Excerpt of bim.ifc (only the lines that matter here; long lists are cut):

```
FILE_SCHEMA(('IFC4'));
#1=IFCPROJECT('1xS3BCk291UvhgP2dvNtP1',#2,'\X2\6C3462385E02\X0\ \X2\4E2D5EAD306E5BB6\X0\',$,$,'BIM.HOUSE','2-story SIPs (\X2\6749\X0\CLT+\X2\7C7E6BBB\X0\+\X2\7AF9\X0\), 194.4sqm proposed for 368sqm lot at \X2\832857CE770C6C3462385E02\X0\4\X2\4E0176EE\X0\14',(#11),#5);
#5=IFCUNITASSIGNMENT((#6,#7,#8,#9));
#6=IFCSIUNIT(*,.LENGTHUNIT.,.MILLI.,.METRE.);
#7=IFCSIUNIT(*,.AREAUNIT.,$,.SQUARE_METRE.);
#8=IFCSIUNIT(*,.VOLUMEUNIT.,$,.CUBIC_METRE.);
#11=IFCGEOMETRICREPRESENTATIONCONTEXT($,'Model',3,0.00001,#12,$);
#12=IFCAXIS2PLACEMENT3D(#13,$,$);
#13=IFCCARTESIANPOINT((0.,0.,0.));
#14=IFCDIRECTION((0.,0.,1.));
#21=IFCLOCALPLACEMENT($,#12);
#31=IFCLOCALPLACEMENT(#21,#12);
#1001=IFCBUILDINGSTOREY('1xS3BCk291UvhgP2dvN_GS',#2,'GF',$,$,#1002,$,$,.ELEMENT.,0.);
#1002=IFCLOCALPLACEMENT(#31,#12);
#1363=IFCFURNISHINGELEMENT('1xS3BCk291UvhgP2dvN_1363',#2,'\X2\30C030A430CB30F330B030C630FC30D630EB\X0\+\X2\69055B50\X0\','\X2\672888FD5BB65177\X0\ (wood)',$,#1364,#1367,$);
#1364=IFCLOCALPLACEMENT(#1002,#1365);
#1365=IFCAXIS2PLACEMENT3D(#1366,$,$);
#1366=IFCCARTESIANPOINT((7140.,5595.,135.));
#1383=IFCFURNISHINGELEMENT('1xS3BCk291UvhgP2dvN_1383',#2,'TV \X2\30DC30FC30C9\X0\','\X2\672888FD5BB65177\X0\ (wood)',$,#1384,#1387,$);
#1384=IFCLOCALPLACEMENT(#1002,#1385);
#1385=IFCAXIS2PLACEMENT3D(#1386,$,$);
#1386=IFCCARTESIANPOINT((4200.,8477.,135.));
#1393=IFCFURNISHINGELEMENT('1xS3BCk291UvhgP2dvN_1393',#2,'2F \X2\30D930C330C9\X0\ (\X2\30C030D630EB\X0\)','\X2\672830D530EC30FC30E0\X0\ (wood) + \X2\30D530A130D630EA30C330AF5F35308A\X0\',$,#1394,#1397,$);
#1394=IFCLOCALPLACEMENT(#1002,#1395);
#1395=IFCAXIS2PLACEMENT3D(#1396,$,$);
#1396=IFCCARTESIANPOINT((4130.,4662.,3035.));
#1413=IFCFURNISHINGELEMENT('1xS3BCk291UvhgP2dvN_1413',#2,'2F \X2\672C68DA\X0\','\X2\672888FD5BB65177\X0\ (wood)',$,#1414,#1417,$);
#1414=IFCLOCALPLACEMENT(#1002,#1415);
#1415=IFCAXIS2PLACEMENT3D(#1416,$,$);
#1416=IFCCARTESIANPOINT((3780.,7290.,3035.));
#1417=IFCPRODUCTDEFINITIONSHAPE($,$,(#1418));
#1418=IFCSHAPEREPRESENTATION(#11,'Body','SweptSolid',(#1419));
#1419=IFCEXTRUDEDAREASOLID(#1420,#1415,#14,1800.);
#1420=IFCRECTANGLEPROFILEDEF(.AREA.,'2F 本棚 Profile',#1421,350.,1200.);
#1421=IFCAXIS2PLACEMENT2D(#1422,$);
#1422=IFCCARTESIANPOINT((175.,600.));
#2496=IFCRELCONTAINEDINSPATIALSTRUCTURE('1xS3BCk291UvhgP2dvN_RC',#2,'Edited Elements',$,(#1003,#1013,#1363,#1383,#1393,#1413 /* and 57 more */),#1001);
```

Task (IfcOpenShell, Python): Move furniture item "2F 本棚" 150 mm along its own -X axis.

```python
import ifcopenshell
import ifcopenshell.api.geometry
import ifcopenshell.util.placement
import ifcopenshell.util.unit

model = ifcopenshell.open("bim.ifc")
unit_scale = ifcopenshell.util.unit.calculate_unit_scale(model)

item = model.by_guid("1xS3BCk291UvhgP2dvN_1413")
matrix = ifcopenshell.util.placement.get_local_placement(item.ObjectPlacement)
matrix[:3, 3] -= matrix[:3, 0] * 0.15 / unit_scale
ifcopenshell.api.geometry.edit_object_placement(model, product=item, matrix=matrix, is_si=False)

print(ifcopenshell.util.placement.get_local_placement(item.ObjectPlacement).round(3) + 0.0)

model.write("bim_v2.ifc")
```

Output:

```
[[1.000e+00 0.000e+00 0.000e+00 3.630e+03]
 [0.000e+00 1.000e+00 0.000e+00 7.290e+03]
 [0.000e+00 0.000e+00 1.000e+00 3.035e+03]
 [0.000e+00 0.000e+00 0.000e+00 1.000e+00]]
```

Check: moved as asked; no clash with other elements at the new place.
